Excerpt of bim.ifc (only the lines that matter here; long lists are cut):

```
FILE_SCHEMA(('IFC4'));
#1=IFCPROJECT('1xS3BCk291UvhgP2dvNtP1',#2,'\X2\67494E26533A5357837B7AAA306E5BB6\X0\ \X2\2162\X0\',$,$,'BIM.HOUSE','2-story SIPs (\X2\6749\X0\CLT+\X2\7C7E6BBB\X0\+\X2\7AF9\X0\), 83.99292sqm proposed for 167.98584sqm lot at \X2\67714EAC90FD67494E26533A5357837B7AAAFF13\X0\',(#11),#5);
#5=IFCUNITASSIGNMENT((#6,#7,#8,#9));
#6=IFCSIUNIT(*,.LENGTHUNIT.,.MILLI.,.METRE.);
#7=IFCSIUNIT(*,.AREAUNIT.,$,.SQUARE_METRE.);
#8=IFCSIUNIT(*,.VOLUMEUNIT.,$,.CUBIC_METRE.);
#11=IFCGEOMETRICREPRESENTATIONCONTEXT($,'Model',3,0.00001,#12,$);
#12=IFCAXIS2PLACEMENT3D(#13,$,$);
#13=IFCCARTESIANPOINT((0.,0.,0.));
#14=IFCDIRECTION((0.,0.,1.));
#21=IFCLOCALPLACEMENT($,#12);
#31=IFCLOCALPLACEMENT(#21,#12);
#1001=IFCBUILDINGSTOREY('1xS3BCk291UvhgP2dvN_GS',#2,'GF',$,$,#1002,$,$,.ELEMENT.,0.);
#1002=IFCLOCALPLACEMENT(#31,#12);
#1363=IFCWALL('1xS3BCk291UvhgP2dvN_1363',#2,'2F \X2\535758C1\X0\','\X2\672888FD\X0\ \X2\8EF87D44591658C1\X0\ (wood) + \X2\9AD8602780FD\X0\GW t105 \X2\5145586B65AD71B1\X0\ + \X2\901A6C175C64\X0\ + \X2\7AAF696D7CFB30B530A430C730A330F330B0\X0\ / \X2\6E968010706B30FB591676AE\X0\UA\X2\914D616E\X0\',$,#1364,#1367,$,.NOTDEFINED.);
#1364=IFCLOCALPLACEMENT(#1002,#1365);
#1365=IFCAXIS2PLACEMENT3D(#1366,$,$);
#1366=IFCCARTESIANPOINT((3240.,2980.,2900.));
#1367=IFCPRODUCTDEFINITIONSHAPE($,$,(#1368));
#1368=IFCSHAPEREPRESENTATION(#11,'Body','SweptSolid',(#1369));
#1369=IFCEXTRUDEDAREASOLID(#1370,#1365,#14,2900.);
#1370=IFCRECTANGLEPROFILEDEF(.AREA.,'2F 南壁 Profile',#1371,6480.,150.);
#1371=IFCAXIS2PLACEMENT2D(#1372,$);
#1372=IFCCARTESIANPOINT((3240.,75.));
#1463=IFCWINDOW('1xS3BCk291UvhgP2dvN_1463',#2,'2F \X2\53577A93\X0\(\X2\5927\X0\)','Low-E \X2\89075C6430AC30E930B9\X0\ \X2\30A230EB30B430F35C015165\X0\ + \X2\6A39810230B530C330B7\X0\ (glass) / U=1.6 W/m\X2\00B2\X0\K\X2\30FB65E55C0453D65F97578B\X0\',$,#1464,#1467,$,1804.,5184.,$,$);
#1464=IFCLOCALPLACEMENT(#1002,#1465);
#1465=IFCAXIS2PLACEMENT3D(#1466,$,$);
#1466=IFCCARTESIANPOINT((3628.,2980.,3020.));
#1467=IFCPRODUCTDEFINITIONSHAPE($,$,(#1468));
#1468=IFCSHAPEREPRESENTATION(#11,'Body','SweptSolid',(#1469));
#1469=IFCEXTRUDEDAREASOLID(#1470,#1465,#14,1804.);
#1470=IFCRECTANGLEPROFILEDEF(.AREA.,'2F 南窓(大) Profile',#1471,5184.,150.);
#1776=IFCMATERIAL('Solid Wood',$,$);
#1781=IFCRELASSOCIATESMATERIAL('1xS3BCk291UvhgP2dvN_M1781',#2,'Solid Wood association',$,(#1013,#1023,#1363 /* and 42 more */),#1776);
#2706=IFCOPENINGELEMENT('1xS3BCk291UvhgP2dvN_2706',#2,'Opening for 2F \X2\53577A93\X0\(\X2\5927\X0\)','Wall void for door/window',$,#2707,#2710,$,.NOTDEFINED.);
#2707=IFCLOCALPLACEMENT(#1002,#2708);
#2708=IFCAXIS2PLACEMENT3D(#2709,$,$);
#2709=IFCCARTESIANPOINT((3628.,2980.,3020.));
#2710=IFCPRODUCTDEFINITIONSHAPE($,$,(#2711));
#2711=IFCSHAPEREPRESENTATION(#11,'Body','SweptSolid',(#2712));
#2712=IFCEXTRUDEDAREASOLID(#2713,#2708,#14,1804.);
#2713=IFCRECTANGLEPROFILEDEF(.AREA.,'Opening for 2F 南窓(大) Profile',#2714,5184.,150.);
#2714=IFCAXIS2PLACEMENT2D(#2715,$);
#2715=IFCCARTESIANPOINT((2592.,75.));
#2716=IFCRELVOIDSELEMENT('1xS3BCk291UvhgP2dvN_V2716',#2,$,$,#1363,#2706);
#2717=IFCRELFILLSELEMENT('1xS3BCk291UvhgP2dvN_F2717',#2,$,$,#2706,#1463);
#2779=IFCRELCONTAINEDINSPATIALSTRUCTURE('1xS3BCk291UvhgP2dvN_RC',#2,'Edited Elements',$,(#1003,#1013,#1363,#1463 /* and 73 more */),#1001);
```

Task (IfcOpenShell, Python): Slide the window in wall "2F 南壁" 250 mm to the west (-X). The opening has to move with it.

```python
import ifcopenshell
import ifcopenshell.api.geometry
import ifcopenshell.util.placement
import ifcopenshell.util.unit

model = ifcopenshell.open("bim.ifc")
unit_scale = ifcopenshell.util.unit.calculate_unit_scale(model)

window = model.by_guid("1xS3BCk291UvhgP2dvN_1463")
opening = window.FillsVoids[0].RelatingOpeningElement
wall = opening.VoidsElements[0].RelatingBuildingElement

wall_matrix = ifcopenshell.util.placement.get_local_placement(wall.ObjectPlacement)
shift = wall_matrix[:3, 0] * -0.25 / unit_scale
before = ifcopenshell.util.placement.get_local_placement(window.ObjectPlacement)[:3, 3].copy()

# The window is not placed relative to its opening, so move both.
for product in (opening, window):
    matrix = ifcopenshell.util.placement.get_local_placement(product.ObjectPlacement)
    matrix[:3, 3] += shift
    ifcopenshell.api.geometry.edit_object_placement(model, product=product, matrix=matrix, is_si=False)

after = ifcopenshell.util.placement.get_local_placement(window.ObjectPlacement)[:3, 3]
print("window moved by", (after - before).round(3) + 0.0)

model.write("bim_updated.ifc")
```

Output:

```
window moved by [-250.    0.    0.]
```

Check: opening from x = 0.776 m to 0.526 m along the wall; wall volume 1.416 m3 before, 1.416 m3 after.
